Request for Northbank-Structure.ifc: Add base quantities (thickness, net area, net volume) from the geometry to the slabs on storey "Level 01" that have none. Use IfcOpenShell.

First a look at what the model holds.

```python
import ifcopenshell
import ifcopenshell.util.element
import ifcopenshell.util.unit

model = ifcopenshell.open("Northbank-Structure.ifc")
print(model.schema)
for unit_type in ("LENGTHUNIT", "AREAUNIT", "VOLUMEUNIT"):
    print(unit_type, ifcopenshell.util.unit.calculate_unit_scale(model, unit_type))
storey = next(s for s in model.by_type("IfcBuildingStorey") if s.Name == "Level 01")
slabs = [e for e in ifcopenshell.util.element.get_decomposition(storey) if e.is_a("IfcSlab")]
for e in sorted(slabs, key=lambda e: e.id()):
    print(e.id(), e.is_a(), e.Name, list(ifcopenshell.util.element.get_psets(e, qtos_only=True)), sep=" | ")
```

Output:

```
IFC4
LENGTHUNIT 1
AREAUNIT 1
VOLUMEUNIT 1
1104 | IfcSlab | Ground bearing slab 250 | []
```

```python
import ifcopenshell
import ifcopenshell.api.pset
import ifcopenshell.geom
import ifcopenshell.util.element
import ifcopenshell.util.shape
import ifcopenshell.util.unit

model = ifcopenshell.open("Northbank-Structure.ifc")
unit_scale = ifcopenshell.util.unit.calculate_unit_scale(model)
area_scale = ifcopenshell.util.unit.calculate_unit_scale(model, "AREAUNIT")
volume_scale = ifcopenshell.util.unit.calculate_unit_scale(model, "VOLUMEUNIT")
settings = ifcopenshell.geom.settings()

storey = next(s for s in model.by_type("IfcBuildingStorey") if s.Name == "Level 01")
slabs = [e for e in ifcopenshell.util.element.get_decomposition(storey) if e.is_a("IfcSlab")]

for e in sorted(slabs, key=lambda e: e.id()):
    if ifcopenshell.util.element.get_psets(e, qtos_only=True, should_inherit=False):
        continue
    # Geometry comes back in metres, in the element's own axes.
    shape = ifcopenshell.geom.create_shape(settings, e)
    values = {
        "Width": ifcopenshell.util.shape.get_z(shape.geometry) / unit_scale,
        "NetArea": ifcopenshell.util.shape.get_footprint_area(shape.geometry) / area_scale,
        "NetVolume": ifcopenshell.util.shape.get_volume(shape.geometry) / volume_scale,
    }
    qto = ifcopenshell.api.pset.add_qto(model, product=e, name="Qto_SlabBaseQuantities")
    ifcopenshell.api.pset.edit_qto(model, qto=qto, properties=values)
    print(e.id(), {k: round(v, 3) for k, v in values.items()})

model.write("Northbank-Structure-out.ifc")
```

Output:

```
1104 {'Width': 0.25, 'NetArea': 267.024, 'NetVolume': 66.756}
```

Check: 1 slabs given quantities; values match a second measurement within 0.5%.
